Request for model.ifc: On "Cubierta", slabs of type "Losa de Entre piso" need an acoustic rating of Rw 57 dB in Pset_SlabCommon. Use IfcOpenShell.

First a look at what the model holds.

```python
import ifcopenshell
import ifcopenshell.util.element

model = ifcopenshell.open("model.ifc")
print(model.schema)
storey = next(s for s in model.by_type("IfcBuildingStorey") if s.Name == "Cubierta")
slabs = [e for e in ifcopenshell.util.element.get_decomposition(storey) if e.is_a("IfcSlab")]
seen = {}
for e in slabs:
    element_type = ifcopenshell.util.element.get_type(e)
    key = (element_type.Name if element_type != e and element_type else None, ifcopenshell.util.element.get_pset(e, "Pset_SlabCommon", "AcousticRating"))
    seen[key] = seen.get(key, 0) + 1
for (name, value), count in sorted(seen.items(), key=str):
    print(count, "x", name, "|", value)
```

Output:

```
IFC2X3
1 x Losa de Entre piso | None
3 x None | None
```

```python
import ifcopenshell
import ifcopenshell.api.pset
import ifcopenshell.util.element

model = ifcopenshell.open("model.ifc")

storey = next(s for s in model.by_type("IfcBuildingStorey") if s.Name == "Cubierta")
slabs = [e for e in ifcopenshell.util.element.get_decomposition(storey) if e.is_a("IfcSlab")]

count = 0
for e in slabs:
    element_type = ifcopenshell.util.element.get_type(e)
    if element_type in (None, e) or element_type.Name != "Losa de Entre piso":
        continue
    # add_pset returns the element's existing set when there is one.
    pset = ifcopenshell.api.pset.add_pset(model, product=e, name="Pset_SlabCommon")
    ifcopenshell.api.pset.edit_pset(model, pset=pset, properties={"AcousticRating": "Rw 57 dB"})
    count += 1

print(count, "slabs updated")

model.write("model_edited.ifc")
```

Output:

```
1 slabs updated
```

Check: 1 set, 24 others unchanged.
